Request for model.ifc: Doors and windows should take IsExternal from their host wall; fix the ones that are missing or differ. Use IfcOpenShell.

First a look at what the model holds.

```python
import ifcopenshell
import ifcopenshell.util.element

model = ifcopenshell.open("model.ifc")
print(model.schema)
seen = {}
for e in model.by_type("IfcDoor") + model.by_type("IfcWindow"):
    if not e.FillsVoids:
        continue
    host = e.FillsVoids[0].RelatingOpeningElement.VoidsElements[0].RelatingBuildingElement
    own = ifcopenshell.util.element.get_pset(e, f"Pset_{e.is_a()[3:].removesuffix('StandardCase')}Common", "IsExternal")
    wall = ifcopenshell.util.element.get_pset(host, "Pset_WallCommon", "IsExternal")
    seen[e.is_a(), own, wall] = seen.get((e.is_a(), own, wall), 0) + 1
for (cls, own, wall), count in sorted(seen.items(), key=str):
    print(count, cls, "IsExternal:", own, "| host wall:", wall)
```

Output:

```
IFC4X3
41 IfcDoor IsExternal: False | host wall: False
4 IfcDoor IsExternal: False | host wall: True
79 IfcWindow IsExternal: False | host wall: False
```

```python
import ifcopenshell
import ifcopenshell.api.pset
import ifcopenshell.util.element

model = ifcopenshell.open("model.ifc")

count = 0
for ifc_class, pset_name in (("IfcDoor", "Pset_DoorCommon"), ("IfcWindow", "Pset_WindowCommon")):
    for e in model.by_type(ifc_class):
        if not e.FillsVoids:
            continue
        host = e.FillsVoids[0].RelatingOpeningElement.VoidsElements[0].RelatingBuildingElement
        external = ifcopenshell.util.element.get_pset(host, "Pset_WallCommon", "IsExternal")
        if external is None or ifcopenshell.util.element.get_pset(e, pset_name, "IsExternal") == external:
            continue
        pset = ifcopenshell.api.pset.add_pset(model, product=e, name=pset_name)
        ifcopenshell.api.pset.edit_pset(model, pset=pset, properties={"IsExternal": external})
        count += 1

print(count, "updated")

model.write("model-out.ifc")
```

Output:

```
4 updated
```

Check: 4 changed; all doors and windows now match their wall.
